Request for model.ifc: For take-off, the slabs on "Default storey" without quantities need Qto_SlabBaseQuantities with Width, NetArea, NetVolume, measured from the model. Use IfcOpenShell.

First a look at what the model holds.

```python
import ifcopenshell
import ifcopenshell.util.element
import ifcopenshell.util.unit

model = ifcopenshell.open("model.ifc")
print(model.schema)
for unit_type in ("LENGTHUNIT", "AREAUNIT", "VOLUMEUNIT"):
    print(unit_type, ifcopenshell.util.unit.calculate_unit_scale(model, unit_type))
storey = next(s for s in model.by_type("IfcBuildingStorey") if s.Name == "Default storey")
slabs = [e for e in ifcopenshell.util.element.get_decomposition(storey) if e.is_a("IfcSlab")]
for e in sorted(slabs, key=lambda e: e.id()):
    print(e.id(), e.is_a(), e.Name, list(ifcopenshell.util.element.get_psets(e, qtos_only=True)), sep=" | ")
```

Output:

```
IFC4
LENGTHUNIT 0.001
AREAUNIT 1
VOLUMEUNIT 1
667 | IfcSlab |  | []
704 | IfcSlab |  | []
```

```python
import ifcopenshell
import ifcopenshell.api.pset
import ifcopenshell.geom
import ifcopenshell.util.element
import ifcopenshell.util.shape
import ifcopenshell.util.unit

model = ifcopenshell.open("model.ifc")
unit_scale = ifcopenshell.util.unit.calculate_unit_scale(model)
area_scale = ifcopenshell.util.unit.calculate_unit_scale(model, "AREAUNIT")
volume_scale = ifcopenshell.util.unit.calculate_unit_scale(model, "VOLUMEUNIT")
settings = ifcopenshell.geom.settings()

storey = next(s for s in model.by_type("IfcBuildingStorey") if s.Name == "Default storey")
slabs = [e for e in ifcopenshell.util.element.get_decomposition(storey) if e.is_a("IfcSlab")]

for e in sorted(slabs, key=lambda e: e.id()):
    if ifcopenshell.util.element.get_psets(e, qtos_only=True, should_inherit=False):
        continue
    # Geometry comes back in metres, in the element's own axes.
    shape = ifcopenshell.geom.create_shape(settings, e)
    values = {
        "Width": ifcopenshell.util.shape.get_z(shape.geometry) / unit_scale,
        "NetArea": ifcopenshell.util.shape.get_footprint_area(shape.geometry) / area_scale,
        "NetVolume": ifcopenshell.util.shape.get_volume(shape.geometry) / volume_scale,
    }
    qto = ifcopenshell.api.pset.add_qto(model, product=e, name="Qto_SlabBaseQuantities")
    ifcopenshell.api.pset.edit_qto(model, qto=qto, properties=values)
    print(e.id(), {k: round(v, 3) for k, v in values.items()})

model.write("model_rev.ifc")
```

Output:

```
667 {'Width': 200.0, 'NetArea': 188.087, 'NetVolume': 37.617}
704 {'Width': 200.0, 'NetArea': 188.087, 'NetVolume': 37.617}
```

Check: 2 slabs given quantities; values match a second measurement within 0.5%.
